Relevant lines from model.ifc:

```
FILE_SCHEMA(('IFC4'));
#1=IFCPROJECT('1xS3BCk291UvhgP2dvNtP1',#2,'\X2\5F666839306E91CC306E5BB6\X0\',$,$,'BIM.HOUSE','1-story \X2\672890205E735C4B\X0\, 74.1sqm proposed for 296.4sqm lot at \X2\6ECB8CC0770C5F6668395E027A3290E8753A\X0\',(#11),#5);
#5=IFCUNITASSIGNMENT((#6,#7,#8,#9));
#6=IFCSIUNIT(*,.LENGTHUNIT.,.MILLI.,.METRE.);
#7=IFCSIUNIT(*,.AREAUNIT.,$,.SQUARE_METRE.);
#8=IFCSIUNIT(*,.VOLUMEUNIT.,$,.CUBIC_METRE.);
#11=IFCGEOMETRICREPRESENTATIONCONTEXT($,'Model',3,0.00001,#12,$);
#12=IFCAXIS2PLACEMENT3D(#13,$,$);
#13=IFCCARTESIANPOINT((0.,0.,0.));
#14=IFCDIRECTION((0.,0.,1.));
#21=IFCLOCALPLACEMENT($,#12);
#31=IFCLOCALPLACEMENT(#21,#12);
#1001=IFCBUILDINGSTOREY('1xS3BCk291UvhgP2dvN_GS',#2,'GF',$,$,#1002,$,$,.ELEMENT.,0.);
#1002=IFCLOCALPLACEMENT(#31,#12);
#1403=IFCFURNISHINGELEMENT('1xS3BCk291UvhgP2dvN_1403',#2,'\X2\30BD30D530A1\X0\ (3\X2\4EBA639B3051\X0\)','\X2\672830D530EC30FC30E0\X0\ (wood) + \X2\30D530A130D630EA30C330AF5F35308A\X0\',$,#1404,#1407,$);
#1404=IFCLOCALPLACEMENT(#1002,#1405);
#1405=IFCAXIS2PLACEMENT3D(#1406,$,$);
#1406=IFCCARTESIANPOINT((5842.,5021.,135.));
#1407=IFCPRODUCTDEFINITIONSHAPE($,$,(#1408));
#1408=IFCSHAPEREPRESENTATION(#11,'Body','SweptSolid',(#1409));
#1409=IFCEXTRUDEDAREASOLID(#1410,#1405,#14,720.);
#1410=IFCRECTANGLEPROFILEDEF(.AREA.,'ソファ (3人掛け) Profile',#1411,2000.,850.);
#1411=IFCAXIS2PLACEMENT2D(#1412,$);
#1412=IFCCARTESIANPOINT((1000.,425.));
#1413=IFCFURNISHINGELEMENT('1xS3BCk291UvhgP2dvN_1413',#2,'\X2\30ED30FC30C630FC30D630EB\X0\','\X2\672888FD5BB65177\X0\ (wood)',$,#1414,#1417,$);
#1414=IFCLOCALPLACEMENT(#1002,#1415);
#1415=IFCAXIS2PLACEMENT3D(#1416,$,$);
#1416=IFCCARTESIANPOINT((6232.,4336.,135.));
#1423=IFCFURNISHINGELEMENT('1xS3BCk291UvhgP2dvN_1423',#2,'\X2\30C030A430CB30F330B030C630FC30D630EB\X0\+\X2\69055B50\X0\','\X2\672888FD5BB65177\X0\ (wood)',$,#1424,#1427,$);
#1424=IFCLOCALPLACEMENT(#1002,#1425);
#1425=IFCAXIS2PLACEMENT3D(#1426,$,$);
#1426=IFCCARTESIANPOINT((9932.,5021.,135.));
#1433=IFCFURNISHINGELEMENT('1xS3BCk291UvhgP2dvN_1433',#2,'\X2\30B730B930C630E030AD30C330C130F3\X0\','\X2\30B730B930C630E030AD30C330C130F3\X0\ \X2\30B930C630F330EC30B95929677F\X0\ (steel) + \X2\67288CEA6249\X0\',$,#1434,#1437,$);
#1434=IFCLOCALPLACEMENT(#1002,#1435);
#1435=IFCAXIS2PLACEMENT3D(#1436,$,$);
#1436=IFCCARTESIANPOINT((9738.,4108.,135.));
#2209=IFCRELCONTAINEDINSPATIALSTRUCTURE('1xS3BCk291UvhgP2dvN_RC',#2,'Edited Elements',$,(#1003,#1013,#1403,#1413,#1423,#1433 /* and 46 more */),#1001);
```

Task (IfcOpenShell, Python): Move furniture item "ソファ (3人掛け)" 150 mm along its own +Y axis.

```python
import ifcopenshell
import ifcopenshell.api.geometry
import ifcopenshell.util.placement
import ifcopenshell.util.unit

model = ifcopenshell.open("model.ifc")
unit_scale = ifcopenshell.util.unit.calculate_unit_scale(model)

item = model.by_id(1403)
matrix = ifcopenshell.util.placement.get_local_placement(item.ObjectPlacement)
matrix[:3, 3] += matrix[:3, 1] * 0.15 / unit_scale
ifcopenshell.api.geometry.edit_object_placement(model, product=item, matrix=matrix, is_si=False)

print(ifcopenshell.util.placement.get_local_placement(item.ObjectPlacement).round(3) + 0.0)

model.write("model_updated.ifc")
```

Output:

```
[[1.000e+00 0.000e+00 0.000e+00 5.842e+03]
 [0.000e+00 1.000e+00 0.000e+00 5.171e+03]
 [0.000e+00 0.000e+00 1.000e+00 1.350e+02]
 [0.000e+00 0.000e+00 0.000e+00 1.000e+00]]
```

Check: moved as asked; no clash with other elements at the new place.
